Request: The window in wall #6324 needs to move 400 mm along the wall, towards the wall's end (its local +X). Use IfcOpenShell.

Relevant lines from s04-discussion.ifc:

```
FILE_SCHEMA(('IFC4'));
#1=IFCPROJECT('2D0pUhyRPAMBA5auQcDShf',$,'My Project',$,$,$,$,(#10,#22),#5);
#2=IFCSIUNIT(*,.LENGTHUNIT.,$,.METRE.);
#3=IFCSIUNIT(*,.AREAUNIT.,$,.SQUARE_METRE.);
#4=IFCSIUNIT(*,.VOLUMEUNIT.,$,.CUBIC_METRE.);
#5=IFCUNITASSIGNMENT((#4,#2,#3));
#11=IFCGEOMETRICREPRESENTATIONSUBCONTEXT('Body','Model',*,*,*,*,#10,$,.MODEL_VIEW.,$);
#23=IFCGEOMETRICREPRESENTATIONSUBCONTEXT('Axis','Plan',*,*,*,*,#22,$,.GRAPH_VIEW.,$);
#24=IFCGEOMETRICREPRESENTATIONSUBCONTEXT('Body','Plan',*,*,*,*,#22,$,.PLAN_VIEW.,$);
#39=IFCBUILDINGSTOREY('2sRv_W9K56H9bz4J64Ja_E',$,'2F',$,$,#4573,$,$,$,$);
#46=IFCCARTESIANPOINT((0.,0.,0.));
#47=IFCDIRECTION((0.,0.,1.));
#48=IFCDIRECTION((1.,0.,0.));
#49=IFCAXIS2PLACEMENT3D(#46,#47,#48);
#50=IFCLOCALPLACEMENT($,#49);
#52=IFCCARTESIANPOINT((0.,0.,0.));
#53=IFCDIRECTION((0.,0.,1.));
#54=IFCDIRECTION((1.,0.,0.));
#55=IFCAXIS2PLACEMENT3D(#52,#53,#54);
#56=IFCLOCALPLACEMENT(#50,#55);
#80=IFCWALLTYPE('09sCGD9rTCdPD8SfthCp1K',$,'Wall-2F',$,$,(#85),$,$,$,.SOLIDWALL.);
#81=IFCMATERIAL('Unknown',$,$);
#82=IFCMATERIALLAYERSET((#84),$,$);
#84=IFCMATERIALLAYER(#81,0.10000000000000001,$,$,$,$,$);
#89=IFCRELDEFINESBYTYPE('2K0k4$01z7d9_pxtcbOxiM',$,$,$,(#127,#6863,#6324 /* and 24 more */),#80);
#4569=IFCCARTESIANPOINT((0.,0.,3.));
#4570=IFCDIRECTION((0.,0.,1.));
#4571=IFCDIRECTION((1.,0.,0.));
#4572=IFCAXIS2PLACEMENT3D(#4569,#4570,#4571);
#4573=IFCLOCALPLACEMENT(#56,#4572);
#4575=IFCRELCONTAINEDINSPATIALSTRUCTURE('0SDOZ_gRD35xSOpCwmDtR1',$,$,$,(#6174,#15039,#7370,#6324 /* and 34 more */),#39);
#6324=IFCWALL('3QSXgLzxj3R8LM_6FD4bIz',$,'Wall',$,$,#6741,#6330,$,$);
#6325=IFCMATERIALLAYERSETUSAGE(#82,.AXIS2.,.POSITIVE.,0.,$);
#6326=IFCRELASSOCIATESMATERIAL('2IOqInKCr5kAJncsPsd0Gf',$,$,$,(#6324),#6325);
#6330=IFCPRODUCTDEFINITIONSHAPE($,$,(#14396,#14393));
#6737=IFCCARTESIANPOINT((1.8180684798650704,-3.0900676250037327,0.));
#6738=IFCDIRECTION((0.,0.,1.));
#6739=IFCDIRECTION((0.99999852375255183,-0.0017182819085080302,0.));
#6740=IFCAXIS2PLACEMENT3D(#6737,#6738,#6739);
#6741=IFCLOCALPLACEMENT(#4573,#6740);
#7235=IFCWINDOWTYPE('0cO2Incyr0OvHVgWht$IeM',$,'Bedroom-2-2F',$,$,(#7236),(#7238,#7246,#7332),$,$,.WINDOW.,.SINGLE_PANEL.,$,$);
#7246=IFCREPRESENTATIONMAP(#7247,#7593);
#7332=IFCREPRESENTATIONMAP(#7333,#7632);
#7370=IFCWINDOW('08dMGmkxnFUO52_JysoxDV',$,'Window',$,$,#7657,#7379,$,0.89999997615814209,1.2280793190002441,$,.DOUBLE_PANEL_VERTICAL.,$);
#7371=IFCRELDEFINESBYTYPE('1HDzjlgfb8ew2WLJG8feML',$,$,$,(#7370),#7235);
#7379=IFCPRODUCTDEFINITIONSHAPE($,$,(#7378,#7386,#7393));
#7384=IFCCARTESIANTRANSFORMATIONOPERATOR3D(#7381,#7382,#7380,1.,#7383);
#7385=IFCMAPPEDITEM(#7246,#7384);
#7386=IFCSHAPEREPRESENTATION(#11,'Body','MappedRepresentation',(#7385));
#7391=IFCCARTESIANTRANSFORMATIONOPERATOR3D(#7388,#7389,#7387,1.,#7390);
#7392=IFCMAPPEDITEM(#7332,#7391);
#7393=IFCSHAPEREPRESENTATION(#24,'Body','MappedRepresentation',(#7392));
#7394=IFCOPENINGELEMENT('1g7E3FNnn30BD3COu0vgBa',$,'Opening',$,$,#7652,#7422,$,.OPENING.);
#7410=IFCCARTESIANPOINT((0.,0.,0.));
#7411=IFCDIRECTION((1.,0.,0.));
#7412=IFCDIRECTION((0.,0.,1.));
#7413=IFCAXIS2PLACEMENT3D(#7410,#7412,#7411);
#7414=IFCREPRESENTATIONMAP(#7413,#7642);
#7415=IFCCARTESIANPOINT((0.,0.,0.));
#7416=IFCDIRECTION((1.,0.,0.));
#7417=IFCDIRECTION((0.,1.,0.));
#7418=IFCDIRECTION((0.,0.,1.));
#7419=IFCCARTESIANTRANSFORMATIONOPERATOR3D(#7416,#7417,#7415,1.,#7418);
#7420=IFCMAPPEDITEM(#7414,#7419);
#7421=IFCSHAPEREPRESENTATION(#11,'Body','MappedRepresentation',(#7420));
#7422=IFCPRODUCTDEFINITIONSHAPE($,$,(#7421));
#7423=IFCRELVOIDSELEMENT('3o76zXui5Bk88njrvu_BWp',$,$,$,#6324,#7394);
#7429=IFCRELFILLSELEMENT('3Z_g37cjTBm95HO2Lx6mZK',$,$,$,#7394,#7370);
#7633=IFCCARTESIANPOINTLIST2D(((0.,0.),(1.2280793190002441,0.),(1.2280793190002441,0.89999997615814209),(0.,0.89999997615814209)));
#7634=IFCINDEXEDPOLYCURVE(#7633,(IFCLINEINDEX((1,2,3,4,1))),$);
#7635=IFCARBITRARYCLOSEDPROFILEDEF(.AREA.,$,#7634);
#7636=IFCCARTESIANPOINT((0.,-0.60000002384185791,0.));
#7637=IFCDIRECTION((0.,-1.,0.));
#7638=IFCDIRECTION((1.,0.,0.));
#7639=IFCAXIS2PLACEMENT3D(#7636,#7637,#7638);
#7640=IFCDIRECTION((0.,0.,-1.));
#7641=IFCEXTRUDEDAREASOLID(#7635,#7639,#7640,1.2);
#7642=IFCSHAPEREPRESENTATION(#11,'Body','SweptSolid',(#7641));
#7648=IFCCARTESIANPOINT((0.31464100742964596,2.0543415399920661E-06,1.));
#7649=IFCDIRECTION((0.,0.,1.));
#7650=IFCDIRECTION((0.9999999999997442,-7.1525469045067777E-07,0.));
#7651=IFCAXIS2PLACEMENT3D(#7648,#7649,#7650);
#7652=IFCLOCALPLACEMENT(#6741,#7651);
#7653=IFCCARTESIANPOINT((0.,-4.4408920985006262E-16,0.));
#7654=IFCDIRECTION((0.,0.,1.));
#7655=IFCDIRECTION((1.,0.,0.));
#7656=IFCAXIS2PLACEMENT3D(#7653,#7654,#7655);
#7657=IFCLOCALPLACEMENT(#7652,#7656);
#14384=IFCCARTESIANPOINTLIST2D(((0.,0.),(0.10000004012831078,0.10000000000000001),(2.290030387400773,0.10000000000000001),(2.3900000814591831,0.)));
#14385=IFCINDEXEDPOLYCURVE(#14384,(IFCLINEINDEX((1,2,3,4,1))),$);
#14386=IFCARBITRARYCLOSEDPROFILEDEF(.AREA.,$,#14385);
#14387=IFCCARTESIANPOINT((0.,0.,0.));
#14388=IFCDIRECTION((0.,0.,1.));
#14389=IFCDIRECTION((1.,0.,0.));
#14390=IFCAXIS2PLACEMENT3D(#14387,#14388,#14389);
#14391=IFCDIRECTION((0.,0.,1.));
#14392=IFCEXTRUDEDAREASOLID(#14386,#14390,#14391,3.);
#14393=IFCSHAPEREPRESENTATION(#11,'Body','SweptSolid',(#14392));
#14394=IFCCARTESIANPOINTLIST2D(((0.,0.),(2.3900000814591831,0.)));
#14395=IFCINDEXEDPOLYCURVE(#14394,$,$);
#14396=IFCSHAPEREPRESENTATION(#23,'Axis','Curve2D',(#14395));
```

```python
import ifcopenshell
import ifcopenshell.api.geometry
import ifcopenshell.util.placement

model = ifcopenshell.open("s04-discussion.ifc")

window = model.by_guid("08dMGmkxnFUO52_JysoxDV")
opening = window.FillsVoids[0].RelatingOpeningElement
wall = opening.VoidsElements[0].RelatingBuildingElement

wall_matrix = ifcopenshell.util.placement.get_local_placement(wall.ObjectPlacement)
shift = wall_matrix[:3, 0] * 0.4
before = ifcopenshell.util.placement.get_local_placement(window.ObjectPlacement)[:3, 3].copy()

# The window is placed relative to its opening, so it follows when the opening moves.
matrix = ifcopenshell.util.placement.get_local_placement(opening.ObjectPlacement)
matrix[:3, 3] += shift
ifcopenshell.api.geometry.edit_object_placement(
    model, product=opening, matrix=matrix, is_si=False, should_transform_children=True
)

after = ifcopenshell.util.placement.get_local_placement(window.ObjectPlacement)[:3, 3]
print("window moved by", (after - before).round(3) + 0.0)

model.write("s04-discussion_updated.ifc")
```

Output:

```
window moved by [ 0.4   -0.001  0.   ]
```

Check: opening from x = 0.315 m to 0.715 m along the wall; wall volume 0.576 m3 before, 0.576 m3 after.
